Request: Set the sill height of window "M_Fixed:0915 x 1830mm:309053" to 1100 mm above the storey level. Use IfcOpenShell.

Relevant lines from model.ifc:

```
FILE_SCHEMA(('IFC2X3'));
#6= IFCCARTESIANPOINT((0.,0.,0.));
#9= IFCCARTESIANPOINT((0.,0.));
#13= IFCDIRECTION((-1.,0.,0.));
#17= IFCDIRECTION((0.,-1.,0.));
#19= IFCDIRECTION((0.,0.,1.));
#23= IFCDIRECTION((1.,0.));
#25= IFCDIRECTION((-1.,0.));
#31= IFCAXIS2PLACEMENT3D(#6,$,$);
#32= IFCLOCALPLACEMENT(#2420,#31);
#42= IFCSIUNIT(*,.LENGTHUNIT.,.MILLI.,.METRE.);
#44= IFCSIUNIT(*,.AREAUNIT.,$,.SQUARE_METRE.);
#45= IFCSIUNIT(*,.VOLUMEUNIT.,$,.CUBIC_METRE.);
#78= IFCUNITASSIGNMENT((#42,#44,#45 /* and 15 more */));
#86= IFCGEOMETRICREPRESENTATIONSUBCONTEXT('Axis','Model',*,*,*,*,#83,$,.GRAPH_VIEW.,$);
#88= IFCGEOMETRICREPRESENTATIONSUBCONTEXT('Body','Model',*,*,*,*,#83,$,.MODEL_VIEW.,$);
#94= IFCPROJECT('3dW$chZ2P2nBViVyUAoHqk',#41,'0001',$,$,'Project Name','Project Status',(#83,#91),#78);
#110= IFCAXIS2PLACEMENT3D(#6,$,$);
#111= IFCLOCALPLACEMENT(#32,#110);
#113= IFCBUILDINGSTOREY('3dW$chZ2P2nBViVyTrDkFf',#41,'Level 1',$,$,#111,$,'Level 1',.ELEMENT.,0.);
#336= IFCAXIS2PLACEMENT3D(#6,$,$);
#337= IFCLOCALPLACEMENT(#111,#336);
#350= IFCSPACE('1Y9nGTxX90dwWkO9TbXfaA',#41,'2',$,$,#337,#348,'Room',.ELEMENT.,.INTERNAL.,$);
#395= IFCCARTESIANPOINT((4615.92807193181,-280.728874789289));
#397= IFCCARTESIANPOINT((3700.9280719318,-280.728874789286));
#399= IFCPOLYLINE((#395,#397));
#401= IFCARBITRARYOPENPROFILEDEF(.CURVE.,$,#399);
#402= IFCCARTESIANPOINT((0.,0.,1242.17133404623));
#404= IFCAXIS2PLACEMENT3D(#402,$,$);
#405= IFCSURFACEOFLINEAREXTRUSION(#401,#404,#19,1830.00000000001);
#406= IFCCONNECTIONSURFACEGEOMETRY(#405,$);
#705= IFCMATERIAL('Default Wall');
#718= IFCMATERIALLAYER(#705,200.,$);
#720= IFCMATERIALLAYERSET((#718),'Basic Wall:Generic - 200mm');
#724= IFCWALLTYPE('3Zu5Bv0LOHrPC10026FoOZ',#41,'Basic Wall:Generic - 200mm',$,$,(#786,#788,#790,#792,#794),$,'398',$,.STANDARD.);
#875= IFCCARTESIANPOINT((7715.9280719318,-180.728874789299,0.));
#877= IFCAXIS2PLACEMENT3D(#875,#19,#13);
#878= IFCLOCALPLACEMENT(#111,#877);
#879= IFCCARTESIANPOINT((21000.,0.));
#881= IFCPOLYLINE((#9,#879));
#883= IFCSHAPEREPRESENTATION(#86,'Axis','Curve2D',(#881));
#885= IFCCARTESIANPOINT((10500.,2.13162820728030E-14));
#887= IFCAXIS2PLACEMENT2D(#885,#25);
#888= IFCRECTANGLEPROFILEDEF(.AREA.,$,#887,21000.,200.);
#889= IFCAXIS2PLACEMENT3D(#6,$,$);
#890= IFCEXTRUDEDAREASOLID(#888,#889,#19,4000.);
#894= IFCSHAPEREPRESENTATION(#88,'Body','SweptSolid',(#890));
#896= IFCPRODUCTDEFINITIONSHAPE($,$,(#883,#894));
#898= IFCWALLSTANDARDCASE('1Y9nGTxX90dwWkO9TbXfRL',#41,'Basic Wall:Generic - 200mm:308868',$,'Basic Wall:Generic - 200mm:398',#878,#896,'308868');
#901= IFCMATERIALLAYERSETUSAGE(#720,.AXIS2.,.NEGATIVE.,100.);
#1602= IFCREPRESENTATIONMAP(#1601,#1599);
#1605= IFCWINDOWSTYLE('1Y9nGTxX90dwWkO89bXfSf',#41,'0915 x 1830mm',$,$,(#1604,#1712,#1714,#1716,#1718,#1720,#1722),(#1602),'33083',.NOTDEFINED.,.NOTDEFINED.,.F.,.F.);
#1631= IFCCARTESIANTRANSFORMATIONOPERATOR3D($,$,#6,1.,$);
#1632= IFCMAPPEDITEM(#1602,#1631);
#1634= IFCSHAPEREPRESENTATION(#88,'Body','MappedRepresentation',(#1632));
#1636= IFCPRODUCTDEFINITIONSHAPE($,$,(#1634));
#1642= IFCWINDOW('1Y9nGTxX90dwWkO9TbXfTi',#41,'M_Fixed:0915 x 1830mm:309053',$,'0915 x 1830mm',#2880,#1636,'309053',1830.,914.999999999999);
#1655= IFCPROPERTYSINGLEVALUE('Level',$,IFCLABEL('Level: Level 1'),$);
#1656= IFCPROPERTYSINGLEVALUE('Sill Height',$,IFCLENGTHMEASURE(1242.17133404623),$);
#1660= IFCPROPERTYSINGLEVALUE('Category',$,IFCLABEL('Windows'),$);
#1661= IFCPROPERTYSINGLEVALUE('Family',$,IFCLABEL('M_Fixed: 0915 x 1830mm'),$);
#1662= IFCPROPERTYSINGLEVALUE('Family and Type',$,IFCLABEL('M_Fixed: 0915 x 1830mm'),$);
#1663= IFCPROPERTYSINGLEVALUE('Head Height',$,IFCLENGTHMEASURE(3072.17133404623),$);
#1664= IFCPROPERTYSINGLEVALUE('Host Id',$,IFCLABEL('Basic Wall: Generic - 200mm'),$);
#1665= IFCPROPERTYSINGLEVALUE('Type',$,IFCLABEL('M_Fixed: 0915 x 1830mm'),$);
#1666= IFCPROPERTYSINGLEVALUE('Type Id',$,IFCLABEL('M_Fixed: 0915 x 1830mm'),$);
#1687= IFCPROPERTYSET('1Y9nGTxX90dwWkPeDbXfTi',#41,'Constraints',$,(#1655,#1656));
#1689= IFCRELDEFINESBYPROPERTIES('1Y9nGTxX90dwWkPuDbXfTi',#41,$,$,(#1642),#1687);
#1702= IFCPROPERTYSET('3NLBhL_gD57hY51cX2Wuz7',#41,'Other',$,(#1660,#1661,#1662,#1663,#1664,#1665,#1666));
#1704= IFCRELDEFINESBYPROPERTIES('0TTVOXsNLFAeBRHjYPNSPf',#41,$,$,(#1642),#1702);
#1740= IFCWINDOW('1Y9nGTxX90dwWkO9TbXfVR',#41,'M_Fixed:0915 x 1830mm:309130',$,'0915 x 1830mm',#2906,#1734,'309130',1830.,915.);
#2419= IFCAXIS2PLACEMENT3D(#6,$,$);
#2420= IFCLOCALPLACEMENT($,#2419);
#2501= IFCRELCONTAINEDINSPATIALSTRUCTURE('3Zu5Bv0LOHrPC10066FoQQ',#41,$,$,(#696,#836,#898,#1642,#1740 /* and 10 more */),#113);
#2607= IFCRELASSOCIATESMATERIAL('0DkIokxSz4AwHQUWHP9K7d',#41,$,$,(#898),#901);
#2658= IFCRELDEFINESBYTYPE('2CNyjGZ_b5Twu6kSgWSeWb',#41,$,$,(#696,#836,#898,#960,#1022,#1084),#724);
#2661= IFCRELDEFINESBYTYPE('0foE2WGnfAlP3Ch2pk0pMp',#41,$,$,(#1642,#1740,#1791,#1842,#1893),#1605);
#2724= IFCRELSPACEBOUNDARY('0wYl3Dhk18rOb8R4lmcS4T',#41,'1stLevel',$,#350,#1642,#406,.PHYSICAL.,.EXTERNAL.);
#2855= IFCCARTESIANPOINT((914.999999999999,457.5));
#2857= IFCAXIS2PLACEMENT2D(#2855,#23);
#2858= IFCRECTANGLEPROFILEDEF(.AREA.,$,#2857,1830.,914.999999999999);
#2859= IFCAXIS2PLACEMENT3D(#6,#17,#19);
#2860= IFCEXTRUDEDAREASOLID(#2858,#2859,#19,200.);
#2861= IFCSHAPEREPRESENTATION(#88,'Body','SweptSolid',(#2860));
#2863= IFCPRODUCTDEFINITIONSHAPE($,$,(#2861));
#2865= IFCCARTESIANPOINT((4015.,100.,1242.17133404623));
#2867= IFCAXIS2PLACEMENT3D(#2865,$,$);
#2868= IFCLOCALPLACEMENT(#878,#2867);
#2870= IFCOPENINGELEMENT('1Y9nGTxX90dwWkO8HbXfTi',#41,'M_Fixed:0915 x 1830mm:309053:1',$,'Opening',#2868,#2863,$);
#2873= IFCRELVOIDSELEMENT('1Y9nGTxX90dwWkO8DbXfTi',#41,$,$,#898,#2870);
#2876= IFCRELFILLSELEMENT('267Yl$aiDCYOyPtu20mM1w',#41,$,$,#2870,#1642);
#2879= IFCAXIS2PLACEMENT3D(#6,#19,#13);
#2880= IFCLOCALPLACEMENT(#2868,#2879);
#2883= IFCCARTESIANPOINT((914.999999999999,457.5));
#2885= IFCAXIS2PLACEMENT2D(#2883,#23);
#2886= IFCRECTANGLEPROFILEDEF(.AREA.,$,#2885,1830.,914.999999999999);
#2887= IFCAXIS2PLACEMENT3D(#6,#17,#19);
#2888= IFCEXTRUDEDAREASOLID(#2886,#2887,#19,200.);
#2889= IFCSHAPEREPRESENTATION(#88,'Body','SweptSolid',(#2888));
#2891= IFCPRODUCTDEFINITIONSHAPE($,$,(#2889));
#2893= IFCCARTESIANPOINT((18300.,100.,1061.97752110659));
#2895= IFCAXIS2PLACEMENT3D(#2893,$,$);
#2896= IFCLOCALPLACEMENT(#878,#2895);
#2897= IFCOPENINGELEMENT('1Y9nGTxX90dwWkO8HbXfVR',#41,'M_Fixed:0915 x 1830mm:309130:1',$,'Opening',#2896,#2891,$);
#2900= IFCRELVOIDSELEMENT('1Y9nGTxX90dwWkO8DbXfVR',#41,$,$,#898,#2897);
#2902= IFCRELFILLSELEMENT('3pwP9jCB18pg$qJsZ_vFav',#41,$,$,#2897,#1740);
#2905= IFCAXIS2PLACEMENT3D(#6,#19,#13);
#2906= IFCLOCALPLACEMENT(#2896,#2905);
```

```python
import numpy as np
import ifcopenshell
import ifcopenshell.api.geometry
import ifcopenshell.api.pset
import ifcopenshell.geom
import ifcopenshell.util.element
import ifcopenshell.util.placement
import ifcopenshell.util.shape
import ifcopenshell.util.unit

model = ifcopenshell.open("model.ifc")
unit_scale = ifcopenshell.util.unit.calculate_unit_scale(model)

window = model.by_guid("1Y9nGTxX90dwWkO9TbXfTi")
opening = window.FillsVoids[0].RelatingOpeningElement
storey = ifcopenshell.util.element.get_container(window, ifc_class="IfcBuildingStorey")
level = ifcopenshell.util.placement.get_local_placement(storey.ObjectPlacement)[2, 3]

# The opening's origin need not be at the sill, so measure its lowest point.
shape = ifcopenshell.geom.create_shape(ifcopenshell.geom.settings(), opening)
bottom = ifcopenshell.util.shape.get_shape_bottom_elevation(shape, shape.geometry) / unit_scale
dz = level + 1100.0 - bottom

shift = np.array([0.0, 0.0, dz])
# The window is placed relative to its opening, so it follows when the opening moves.
matrix = ifcopenshell.util.placement.get_local_placement(opening.ObjectPlacement)
matrix[:3, 3] += shift
ifcopenshell.api.geometry.edit_object_placement(
    model, product=opening, matrix=matrix, is_si=False, should_transform_children=True
)

# Space boundary surfaces are stored in each space's coordinates; move them too.
for rel in window.ProvidesBoundaries:
    if not rel.ConnectionGeometry:
        continue
    surface = rel.ConnectionGeometry.SurfaceOnRelatingElement
    space_matrix = ifcopenshell.util.placement.get_local_placement(rel.RelatingSpace.ObjectPlacement)
    point = np.array(surface.Position.Location.Coordinates) + space_matrix[:3, :3].T @ shift
    surface.Position = model.createIfcAxis2Placement3D(
        model.createIfcCartesianPoint(point.tolist()), surface.Position.Axis, surface.Position.RefDirection
    )

# Keep the stored heights in step.
pset = model.by_id(ifcopenshell.util.element.get_pset(window, "Constraints", should_inherit=False)["id"])
ifcopenshell.api.pset.edit_pset(model, pset=pset, properties={
    "Sill Height": model.create_entity("IfcLengthMeasure", ifcopenshell.util.element.get_pset(window, "Constraints", "Sill Height") + dz),
})
pset = model.by_id(ifcopenshell.util.element.get_pset(window, "Other", should_inherit=False)["id"])
ifcopenshell.api.pset.edit_pset(model, pset=pset, properties={
    "Head Height": model.create_entity("IfcLengthMeasure", ifcopenshell.util.element.get_pset(window, "Other", "Head Height") + dz),
})

print(f"moved by {dz * unit_scale:+.3f} m")

model.write("model_edited.ifc")
```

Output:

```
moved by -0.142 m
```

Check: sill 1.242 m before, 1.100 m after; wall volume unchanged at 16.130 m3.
